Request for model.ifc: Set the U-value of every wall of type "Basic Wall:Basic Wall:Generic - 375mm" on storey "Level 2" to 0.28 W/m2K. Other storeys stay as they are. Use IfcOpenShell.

First a look at what the model holds.

```python
import ifcopenshell
import ifcopenshell.util.element

model = ifcopenshell.open("model.ifc")
print(model.schema)
storey = next(s for s in model.by_type("IfcBuildingStorey") if s.Name == "Level 2")
walls = [e for e in ifcopenshell.util.element.get_decomposition(storey) if e.is_a("IfcWall")]
seen = {}
for e in walls:
    element_type = ifcopenshell.util.element.get_type(e)
    key = (element_type.Name if element_type != e and element_type else None, ifcopenshell.util.element.get_pset(e, "Pset_WallCommon", "ThermalTransmittance"))
    seen[key] = seen.get(key, 0) + 1
for (name, value), count in sorted(seen.items(), key=str):
    print(count, "x", name, "|", value)
```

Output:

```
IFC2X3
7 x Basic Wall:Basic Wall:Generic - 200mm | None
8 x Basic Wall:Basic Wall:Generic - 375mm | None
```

```python
import ifcopenshell
import ifcopenshell.api.pset
import ifcopenshell.util.element

model = ifcopenshell.open("model.ifc")

storey = next(s for s in model.by_type("IfcBuildingStorey") if s.Name == "Level 2")
walls = [e for e in ifcopenshell.util.element.get_decomposition(storey) if e.is_a("IfcWall")]

count = 0
for e in walls:
    element_type = ifcopenshell.util.element.get_type(e)
    if element_type in (None, e) or element_type.Name != "Basic Wall:Basic Wall:Generic - 375mm":
        continue
    # add_pset returns the element's existing set when there is one.
    pset = ifcopenshell.api.pset.add_pset(model, product=e, name="Pset_WallCommon")
    ifcopenshell.api.pset.edit_pset(model, pset=pset, properties={"ThermalTransmittance": 0.28})
    count += 1

print(count, "walls updated")

model.write("model_edited.ifc")
```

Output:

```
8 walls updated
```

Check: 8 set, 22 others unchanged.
